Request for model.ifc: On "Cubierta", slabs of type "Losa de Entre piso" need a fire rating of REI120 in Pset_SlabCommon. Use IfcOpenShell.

First a look at what the model holds.

```python
import ifcopenshell
import ifcopenshell.util.element

model = ifcopenshell.open("model.ifc")
print(model.schema)
storey = next(s for s in model.by_type("IfcBuildingStorey") if s.Name == "Cubierta")
slabs = [e for e in ifcopenshell.util.element.get_decomposition(storey) if e.is_a("IfcSlab")]
seen = {}
for e in slabs:
    element_type = ifcopenshell.util.element.get_type(e)
    key = (element_type.Name if element_type != e and element_type else None, ifcopenshell.util.element.get_pset(e, "Pset_SlabCommon", "FireRating"))
    seen[key] = seen.get(key, 0) + 1
for (name, value), count in sorted(seen.items(), key=str):
    print(count, "x", name, "|", value)
```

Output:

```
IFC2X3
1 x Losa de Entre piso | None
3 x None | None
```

```python
import ifcopenshell
import ifcopenshell.api.pset
import ifcopenshell.util.element

model = ifcopenshell.open("model.ifc")

storey = next(s for s in model.by_type("IfcBuildingStorey") if s.Name == "Cubierta")
slabs = [e for e in ifcopenshell.util.element.get_decomposition(storey) if e.is_a("IfcSlab")]

count = 0
for e in slabs:
    element_type = ifcopenshell.util.element.get_type(e)
    if element_type in (None, e) or element_type.Name != "Losa de Entre piso":
        continue
    # add_pset returns the element's existing set when there is one.
    pset = ifcopenshell.api.pset.add_pset(model, product=e, name="Pset_SlabCommon")
    ifcopenshell.api.pset.edit_pset(model, pset=pset, properties={"FireRating": "REI120"})
    count += 1

print(count, "slabs updated")

model.write("model-out.ifc")
```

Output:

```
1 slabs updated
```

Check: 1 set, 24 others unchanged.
